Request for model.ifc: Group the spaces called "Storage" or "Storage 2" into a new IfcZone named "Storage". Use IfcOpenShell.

First a look at what the model holds.

```python
import ifcopenshell

model = ifcopenshell.open("model.ifc")
print(model.schema)
seen = {}
for space in model.by_type("IfcSpace"):
    seen[space.LongName] = seen.get(space.LongName, 0) + 1
for name, count in sorted(seen.items(), key=str):
    print(count, "x", name)
print("zones:", [z.Name for z in model.by_type("IfcZone")][:20])
```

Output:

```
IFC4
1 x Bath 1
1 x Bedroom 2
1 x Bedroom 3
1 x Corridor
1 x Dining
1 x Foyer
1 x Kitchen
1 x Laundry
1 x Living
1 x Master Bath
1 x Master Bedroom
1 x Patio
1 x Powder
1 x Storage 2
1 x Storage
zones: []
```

```python
import ifcopenshell
import ifcopenshell.api.group
import ifcopenshell.api.root

model = ifcopenshell.open("model.ifc")

names = {"Storage", "Storage 2"}
spaces = [s for s in model.by_type("IfcSpace") if s.LongName in names]

zone = ifcopenshell.api.root.create_entity(model, ifc_class="IfcZone", name="Storage")
ifcopenshell.api.group.assign_group(model, products=spaces, group=zone)
print(len(spaces), "spaces in", zone.Name)

model.write("model_rev.ifc")
```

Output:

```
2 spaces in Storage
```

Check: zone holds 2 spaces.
